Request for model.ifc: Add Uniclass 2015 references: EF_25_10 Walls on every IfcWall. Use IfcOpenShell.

First a look at what the model holds.

```python
import ifcopenshell

model = ifcopenshell.open("model.ifc")
print(model.schema)
print("classifications:", [c.Name for c in model.by_type("IfcClassification")])
for ifc_class in ("IfcDoor", "IfcRoof", "IfcStair", "IfcWall", "IfcWindow"):
    print(ifc_class, len(model.by_type(ifc_class)))
```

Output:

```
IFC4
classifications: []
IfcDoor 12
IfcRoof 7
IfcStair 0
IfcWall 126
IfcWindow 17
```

```python
import ifcopenshell
import ifcopenshell.api.classification

model = ifcopenshell.open("model.ifc")

system = ifcopenshell.api.classification.add_classification(model, classification="Uniclass 2015")

codes = {
    "IfcWall": ("EF_25_10", "Walls"),
}
for ifc_class, (code, name) in codes.items():
    products = model.by_type(ifc_class)
    ifcopenshell.api.classification.add_reference(
        model, products=products, classification=system, identification=code, name=name
    )
    print(code, len(products))

model.write("model_v2.ifc")
```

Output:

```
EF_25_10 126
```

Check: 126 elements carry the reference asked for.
